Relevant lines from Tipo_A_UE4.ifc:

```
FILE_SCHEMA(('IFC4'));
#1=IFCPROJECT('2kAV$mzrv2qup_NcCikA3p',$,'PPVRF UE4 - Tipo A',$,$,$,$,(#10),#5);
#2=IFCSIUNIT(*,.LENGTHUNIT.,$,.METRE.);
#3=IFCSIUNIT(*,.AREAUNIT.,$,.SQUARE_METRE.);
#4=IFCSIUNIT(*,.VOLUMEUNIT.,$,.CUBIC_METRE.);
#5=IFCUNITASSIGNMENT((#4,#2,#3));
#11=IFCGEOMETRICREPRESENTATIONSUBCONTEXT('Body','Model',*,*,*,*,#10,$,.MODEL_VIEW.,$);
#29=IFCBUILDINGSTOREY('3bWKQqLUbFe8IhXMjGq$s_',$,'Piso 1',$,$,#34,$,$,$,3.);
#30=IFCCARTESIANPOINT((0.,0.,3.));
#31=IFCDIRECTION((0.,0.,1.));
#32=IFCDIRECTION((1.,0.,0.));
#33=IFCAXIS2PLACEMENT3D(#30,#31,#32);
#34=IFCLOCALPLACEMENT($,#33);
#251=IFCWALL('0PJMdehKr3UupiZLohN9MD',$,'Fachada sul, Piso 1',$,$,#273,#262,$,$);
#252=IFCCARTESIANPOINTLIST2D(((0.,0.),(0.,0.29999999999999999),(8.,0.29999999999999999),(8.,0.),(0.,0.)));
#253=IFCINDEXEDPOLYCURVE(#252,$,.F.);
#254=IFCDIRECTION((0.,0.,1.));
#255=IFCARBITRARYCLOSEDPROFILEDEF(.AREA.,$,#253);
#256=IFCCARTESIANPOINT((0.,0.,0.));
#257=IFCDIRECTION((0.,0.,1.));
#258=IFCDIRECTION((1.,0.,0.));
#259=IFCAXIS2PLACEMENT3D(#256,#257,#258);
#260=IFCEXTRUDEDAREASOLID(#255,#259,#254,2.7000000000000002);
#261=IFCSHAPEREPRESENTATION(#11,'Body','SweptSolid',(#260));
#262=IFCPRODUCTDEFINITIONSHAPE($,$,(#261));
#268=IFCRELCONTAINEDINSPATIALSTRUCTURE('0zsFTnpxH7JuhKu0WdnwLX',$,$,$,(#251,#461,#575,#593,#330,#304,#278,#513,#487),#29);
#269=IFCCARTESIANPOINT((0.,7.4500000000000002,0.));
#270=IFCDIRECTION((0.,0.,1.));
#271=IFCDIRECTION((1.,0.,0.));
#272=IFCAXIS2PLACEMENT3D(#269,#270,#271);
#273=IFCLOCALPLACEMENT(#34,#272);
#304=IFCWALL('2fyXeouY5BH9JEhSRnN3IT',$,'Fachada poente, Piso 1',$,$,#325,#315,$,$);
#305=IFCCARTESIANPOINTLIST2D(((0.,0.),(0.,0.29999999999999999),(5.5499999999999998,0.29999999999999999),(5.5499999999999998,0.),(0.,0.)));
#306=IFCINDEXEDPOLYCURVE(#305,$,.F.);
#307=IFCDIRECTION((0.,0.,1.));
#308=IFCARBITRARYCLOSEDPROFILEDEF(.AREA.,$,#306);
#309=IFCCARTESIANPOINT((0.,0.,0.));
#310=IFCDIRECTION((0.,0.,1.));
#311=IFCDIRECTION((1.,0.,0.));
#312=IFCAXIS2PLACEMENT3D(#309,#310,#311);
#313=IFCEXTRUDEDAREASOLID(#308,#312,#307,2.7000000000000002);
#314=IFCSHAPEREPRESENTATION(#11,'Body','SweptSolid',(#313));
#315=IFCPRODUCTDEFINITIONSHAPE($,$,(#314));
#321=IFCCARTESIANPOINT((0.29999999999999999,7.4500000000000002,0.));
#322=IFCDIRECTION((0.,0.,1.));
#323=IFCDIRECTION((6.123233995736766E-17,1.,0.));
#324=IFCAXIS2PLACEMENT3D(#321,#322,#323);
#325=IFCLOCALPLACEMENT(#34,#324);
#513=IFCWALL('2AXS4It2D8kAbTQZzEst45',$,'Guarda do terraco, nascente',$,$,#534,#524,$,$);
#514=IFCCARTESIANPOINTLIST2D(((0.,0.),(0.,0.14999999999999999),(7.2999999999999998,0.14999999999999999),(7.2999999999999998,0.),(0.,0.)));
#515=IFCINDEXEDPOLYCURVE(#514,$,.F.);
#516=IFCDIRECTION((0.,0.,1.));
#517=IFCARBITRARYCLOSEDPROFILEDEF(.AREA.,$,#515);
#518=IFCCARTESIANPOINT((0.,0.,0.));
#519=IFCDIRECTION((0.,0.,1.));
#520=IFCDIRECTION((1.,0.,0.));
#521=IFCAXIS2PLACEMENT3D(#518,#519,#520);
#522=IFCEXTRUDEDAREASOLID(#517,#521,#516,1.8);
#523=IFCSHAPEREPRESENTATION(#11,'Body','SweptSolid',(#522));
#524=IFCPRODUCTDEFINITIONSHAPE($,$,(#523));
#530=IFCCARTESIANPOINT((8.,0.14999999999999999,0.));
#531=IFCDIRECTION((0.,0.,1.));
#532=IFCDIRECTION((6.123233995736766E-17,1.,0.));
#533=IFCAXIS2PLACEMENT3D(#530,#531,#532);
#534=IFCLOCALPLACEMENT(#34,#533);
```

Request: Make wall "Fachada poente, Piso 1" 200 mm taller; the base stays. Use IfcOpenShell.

```python
import ifcopenshell
import ifcopenshell.geom
import ifcopenshell.util.representation
import ifcopenshell.util.shape
import ifcopenshell.util.unit

model = ifcopenshell.open("Tipo_A_UE4.ifc")
unit_scale = ifcopenshell.util.unit.calculate_unit_scale(model)
settings = ifcopenshell.geom.settings()


def volume(element):
    """Net volume in cubic metres, openings subtracted."""
    shape = ifcopenshell.geom.create_shape(settings, element)
    return ifcopenshell.util.shape.get_volume(shape.geometry)


wall = model.by_id(304)
before = volume(wall)

body = ifcopenshell.util.representation.get_representation(wall, "Model", "Body")
solid = body.Items[0]
old_height = solid.Depth
solid.Depth += 0.2 / unit_scale
after = volume(wall)

print(f"height {old_height:g} -> {solid.Depth:g}, volume {before:.3f} -> {after:.3f} m3")

model.write("Tipo_A_UE4_updated.ifc")
```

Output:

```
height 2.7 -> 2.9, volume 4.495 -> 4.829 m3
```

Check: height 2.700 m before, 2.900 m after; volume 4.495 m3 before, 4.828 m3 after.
